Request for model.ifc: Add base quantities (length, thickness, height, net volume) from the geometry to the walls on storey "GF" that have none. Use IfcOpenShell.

First a look at what the model holds.

```python
import ifcopenshell
import ifcopenshell.util.element
import ifcopenshell.util.unit

model = ifcopenshell.open("model.ifc")
print(model.schema)
for unit_type in ("LENGTHUNIT", "AREAUNIT", "VOLUMEUNIT"):
    print(unit_type, ifcopenshell.util.unit.calculate_unit_scale(model, unit_type))
storey = next(s for s in model.by_type("IfcBuildingStorey") if s.Name == "GF")
walls = [e for e in ifcopenshell.util.element.get_decomposition(storey) if e.is_a("IfcWall")]
for e in sorted(walls, key=lambda e: e.id()):
    print(e.id(), e.is_a(), e.Name, list(ifcopenshell.util.element.get_psets(e, qtos_only=True)), sep=" | ")
```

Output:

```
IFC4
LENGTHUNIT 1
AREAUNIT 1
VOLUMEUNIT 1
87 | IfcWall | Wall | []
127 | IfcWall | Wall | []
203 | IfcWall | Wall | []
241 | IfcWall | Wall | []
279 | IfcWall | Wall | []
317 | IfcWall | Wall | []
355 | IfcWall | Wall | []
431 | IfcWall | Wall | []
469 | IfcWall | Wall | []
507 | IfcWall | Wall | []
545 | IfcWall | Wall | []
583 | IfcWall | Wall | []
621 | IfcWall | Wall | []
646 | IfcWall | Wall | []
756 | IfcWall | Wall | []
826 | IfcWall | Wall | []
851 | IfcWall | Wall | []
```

```python
import ifcopenshell
import ifcopenshell.api.pset
import ifcopenshell.geom
import ifcopenshell.util.element
import ifcopenshell.util.shape
import ifcopenshell.util.unit

model = ifcopenshell.open("model.ifc")
unit_scale = ifcopenshell.util.unit.calculate_unit_scale(model)
volume_scale = ifcopenshell.util.unit.calculate_unit_scale(model, "VOLUMEUNIT")
settings = ifcopenshell.geom.settings()

storey = next(s for s in model.by_type("IfcBuildingStorey") if s.Name == "GF")
walls = [e for e in ifcopenshell.util.element.get_decomposition(storey) if e.is_a("IfcWall")]

for e in sorted(walls, key=lambda e: e.id()):
    if ifcopenshell.util.element.get_psets(e, qtos_only=True, should_inherit=False):
        continue
    # Geometry comes back in metres, in the element's own axes.
    shape = ifcopenshell.geom.create_shape(settings, e)
    values = {
        "Length": ifcopenshell.util.shape.get_x(shape.geometry) / unit_scale,
        "Width": ifcopenshell.util.shape.get_y(shape.geometry) / unit_scale,
        "Height": ifcopenshell.util.shape.get_z(shape.geometry) / unit_scale,
        "NetVolume": ifcopenshell.util.shape.get_volume(shape.geometry) / volume_scale,
    }
    qto = ifcopenshell.api.pset.add_qto(model, product=e, name="Qto_WallBaseQuantities")
    ifcopenshell.api.pset.edit_qto(model, qto=qto, properties=values)
    print(e.id(), {k: round(v, 3) for k, v in values.items()})

model.write("model-out.ifc")
```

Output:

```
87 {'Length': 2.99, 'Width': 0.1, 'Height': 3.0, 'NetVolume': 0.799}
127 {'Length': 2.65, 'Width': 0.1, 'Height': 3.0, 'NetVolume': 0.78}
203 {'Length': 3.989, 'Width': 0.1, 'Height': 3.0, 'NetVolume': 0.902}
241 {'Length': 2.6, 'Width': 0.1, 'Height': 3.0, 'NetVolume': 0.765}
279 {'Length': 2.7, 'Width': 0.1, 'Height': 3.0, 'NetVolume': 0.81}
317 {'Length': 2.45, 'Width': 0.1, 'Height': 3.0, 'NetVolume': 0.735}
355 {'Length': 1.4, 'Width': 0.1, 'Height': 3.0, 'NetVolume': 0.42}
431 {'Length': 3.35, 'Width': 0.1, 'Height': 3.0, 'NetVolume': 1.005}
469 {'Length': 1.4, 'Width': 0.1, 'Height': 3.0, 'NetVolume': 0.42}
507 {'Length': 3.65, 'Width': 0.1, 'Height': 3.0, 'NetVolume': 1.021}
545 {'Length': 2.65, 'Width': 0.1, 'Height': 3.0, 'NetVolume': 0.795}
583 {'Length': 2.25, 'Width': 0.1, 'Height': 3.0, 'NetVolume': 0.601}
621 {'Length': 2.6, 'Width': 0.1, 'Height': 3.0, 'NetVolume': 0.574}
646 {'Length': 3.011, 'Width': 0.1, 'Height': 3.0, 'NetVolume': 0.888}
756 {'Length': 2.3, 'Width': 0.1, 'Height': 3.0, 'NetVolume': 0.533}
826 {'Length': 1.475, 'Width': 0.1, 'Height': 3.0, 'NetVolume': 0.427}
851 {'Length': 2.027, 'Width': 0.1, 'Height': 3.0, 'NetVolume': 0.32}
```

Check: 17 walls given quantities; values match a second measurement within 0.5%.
